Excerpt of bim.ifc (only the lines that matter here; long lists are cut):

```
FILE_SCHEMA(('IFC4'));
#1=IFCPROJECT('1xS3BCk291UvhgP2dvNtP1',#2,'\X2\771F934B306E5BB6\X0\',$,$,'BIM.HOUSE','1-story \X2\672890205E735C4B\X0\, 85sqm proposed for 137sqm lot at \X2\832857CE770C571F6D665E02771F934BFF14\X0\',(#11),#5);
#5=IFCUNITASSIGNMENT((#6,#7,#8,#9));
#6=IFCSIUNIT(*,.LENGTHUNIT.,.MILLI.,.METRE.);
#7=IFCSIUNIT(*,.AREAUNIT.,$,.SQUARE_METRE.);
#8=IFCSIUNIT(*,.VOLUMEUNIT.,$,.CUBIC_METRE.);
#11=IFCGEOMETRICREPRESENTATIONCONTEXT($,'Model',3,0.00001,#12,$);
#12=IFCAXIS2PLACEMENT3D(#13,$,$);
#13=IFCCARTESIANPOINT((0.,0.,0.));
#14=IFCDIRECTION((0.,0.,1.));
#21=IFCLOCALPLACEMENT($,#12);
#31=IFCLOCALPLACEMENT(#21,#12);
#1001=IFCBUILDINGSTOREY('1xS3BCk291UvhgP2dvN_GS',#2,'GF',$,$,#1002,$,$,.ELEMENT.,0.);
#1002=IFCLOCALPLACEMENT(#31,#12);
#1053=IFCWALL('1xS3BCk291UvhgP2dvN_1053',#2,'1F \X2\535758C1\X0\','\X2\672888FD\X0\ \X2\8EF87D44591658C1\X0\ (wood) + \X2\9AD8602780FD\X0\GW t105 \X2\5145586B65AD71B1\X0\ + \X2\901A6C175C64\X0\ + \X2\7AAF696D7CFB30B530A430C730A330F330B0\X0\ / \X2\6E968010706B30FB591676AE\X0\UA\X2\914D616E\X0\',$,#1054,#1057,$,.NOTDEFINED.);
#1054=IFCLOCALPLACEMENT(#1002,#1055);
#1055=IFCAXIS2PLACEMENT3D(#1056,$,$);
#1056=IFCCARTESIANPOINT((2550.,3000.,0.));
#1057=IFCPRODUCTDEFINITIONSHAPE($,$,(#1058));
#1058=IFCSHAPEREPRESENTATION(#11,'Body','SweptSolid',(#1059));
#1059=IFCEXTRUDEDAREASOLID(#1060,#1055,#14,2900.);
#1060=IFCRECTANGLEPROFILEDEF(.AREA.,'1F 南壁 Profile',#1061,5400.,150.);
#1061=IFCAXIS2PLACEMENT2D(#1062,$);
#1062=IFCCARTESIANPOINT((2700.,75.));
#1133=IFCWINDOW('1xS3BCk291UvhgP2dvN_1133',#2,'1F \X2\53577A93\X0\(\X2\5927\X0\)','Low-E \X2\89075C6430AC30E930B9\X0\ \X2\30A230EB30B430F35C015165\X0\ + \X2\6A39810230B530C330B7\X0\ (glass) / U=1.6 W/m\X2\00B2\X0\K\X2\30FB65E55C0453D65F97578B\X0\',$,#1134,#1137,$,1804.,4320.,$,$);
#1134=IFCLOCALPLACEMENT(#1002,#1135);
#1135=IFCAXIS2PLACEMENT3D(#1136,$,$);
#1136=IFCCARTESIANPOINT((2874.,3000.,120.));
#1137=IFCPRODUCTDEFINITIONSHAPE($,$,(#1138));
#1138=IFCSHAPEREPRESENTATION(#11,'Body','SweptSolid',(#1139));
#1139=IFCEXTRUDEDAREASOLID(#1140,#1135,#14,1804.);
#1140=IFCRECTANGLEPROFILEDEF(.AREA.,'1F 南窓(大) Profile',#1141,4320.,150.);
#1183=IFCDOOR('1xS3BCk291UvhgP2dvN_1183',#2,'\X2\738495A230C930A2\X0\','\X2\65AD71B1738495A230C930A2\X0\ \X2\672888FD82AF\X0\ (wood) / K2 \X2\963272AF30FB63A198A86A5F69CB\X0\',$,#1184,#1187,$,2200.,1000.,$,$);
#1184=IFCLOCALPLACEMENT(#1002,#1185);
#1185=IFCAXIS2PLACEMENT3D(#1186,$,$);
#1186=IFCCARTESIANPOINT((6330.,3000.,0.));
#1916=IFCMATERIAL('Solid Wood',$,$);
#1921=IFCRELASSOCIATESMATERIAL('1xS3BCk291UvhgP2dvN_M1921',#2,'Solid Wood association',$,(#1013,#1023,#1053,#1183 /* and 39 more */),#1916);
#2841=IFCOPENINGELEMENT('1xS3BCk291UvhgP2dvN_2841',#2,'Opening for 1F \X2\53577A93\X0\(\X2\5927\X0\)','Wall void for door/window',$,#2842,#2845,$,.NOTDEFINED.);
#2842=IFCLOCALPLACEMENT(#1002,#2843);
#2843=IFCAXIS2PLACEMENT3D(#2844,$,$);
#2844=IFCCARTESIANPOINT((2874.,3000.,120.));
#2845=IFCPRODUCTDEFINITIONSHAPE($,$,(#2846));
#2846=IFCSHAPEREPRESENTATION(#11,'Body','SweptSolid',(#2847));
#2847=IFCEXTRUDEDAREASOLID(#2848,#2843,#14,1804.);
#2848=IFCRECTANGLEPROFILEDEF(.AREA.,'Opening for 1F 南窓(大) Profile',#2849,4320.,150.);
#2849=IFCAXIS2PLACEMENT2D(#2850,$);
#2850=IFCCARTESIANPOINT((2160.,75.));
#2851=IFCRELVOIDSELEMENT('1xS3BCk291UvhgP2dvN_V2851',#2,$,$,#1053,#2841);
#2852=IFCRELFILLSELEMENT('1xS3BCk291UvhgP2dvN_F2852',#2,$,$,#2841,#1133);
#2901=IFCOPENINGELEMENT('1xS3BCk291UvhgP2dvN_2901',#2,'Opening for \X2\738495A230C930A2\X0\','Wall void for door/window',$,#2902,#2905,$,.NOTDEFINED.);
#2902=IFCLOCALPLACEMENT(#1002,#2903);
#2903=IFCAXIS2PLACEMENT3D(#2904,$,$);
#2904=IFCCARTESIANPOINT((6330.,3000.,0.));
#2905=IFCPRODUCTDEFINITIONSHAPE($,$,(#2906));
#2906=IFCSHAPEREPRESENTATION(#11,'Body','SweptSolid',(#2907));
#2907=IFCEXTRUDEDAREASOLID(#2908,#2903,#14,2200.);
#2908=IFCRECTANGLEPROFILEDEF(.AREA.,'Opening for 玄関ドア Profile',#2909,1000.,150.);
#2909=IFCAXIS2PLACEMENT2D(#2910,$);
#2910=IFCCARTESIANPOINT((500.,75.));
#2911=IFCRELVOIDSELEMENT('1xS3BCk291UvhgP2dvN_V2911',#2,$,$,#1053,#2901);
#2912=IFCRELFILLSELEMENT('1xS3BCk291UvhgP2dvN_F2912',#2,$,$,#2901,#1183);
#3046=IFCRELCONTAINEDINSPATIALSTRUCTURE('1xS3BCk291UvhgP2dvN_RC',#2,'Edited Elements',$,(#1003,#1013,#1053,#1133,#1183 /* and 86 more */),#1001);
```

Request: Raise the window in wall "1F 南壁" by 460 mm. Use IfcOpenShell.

```python
import numpy as np
import ifcopenshell
import ifcopenshell.api.geometry
import ifcopenshell.util.placement
import ifcopenshell.util.unit

model = ifcopenshell.open("bim.ifc")
unit_scale = ifcopenshell.util.unit.calculate_unit_scale(model)

window = model.by_guid("1xS3BCk291UvhgP2dvN_1133")
opening = window.FillsVoids[0].RelatingOpeningElement
dz = 0.46 / unit_scale

shift = np.array([0.0, 0.0, dz])
# The window is not placed relative to its opening, so move both.
for product in (opening, window):
    matrix = ifcopenshell.util.placement.get_local_placement(product.ObjectPlacement)
    matrix[:3, 3] += shift
    ifcopenshell.api.geometry.edit_object_placement(model, product=product, matrix=matrix, is_si=False)

print(f"moved by {dz * unit_scale:+.3f} m")

model.write("bim_v2.ifc")
```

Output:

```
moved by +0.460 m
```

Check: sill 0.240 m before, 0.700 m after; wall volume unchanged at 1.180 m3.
